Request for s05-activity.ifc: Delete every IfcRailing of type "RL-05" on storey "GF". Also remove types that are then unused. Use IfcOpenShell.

First a look at what the model holds.

```python
import ifcopenshell
import ifcopenshell.util.element

model = ifcopenshell.open("s05-activity.ifc")
print(model.schema)
storey = next(s for s in model.by_type("IfcBuildingStorey") if s.Name == "GF")
railings = [e for e in ifcopenshell.util.element.get_decomposition(storey) if e.is_a("IfcRailing")]
seen = {}
for e in railings:
    element_type = ifcopenshell.util.element.get_type(e)
    name = element_type.Name if element_type not in (None, e) else None
    seen[name] = seen.get(name, 0) + 1
for name, count in sorted(seen.items(), key=str):
    print(count, "x", name)
```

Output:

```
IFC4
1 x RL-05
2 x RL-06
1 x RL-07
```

```python
import ifcopenshell
import ifcopenshell.api.root
import ifcopenshell.util.element

model = ifcopenshell.open("s05-activity.ifc")

storey = next(s for s in model.by_type("IfcBuildingStorey") if s.Name == "GF")
railings = [e for e in ifcopenshell.util.element.get_decomposition(storey) if e.is_a("IfcRailing")]
targets = [e for e in railings if (t := ifcopenshell.util.element.get_type(e)) not in (None, e) and t.Name == "RL-05"]
types = {ifcopenshell.util.element.get_type(e) for e in targets} - {None, *targets}

for e in targets:
    ifcopenshell.api.root.remove_product(model, product=e)
print(len(targets), "removed")

unused = [t for t in types if not ifcopenshell.util.element.get_types(t)]
for t in unused:
    ifcopenshell.api.root.remove_product(model, product=t)
print(len(unused), "unused types removed")

model.write("s05-activity_edited.ifc")
```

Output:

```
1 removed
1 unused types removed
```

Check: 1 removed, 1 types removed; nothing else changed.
